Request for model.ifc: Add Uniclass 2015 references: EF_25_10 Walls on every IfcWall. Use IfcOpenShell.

First a look at what the model holds.

```python
import ifcopenshell

model = ifcopenshell.open("model.ifc")
print(model.schema)
print("classifications:", [c.Name for c in model.by_type("IfcClassification")])
for ifc_class in ("IfcDoor", "IfcRoof", "IfcStair", "IfcWall", "IfcWindow"):
    print(ifc_class, len(model.by_type(ifc_class)))
```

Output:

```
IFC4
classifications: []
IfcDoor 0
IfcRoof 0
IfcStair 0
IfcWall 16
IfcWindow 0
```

```python
import ifcopenshell
import ifcopenshell.api.classification

model = ifcopenshell.open("model.ifc")

system = ifcopenshell.api.classification.add_classification(model, classification="Uniclass 2015")

codes = {
    "IfcWall": ("EF_25_10", "Walls"),
}
for ifc_class, (code, name) in codes.items():
    products = model.by_type(ifc_class)
    ifcopenshell.api.classification.add_reference(
        model, products=products, classification=system, identification=code, name=name
    )
    print(code, len(products))

model.write("model_rev.ifc")
```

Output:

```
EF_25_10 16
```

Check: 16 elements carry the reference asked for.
